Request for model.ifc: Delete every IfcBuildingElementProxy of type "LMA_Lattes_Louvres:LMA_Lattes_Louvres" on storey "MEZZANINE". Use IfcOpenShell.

First a look at what the model holds.

```python
import ifcopenshell
import ifcopenshell.util.element

model = ifcopenshell.open("model.ifc")
print(model.schema)
storey = next(s for s in model.by_type("IfcBuildingStorey") if s.Name == "MEZZANINE")
proxies = [e for e in ifcopenshell.util.element.get_decomposition(storey) if e.is_a("IfcBuildingElementProxy")]
seen = {}
for e in proxies:
    element_type = ifcopenshell.util.element.get_type(e)
    name = element_type.Name if element_type not in (None, e) else None
    seen[name] = seen.get(name, 0) + 1
for name, count in sorted(seen.items(), key=str):
    print(count, "x", name)
```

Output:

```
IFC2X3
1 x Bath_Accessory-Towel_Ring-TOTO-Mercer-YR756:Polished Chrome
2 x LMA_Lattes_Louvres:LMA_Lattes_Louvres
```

```python
import ifcopenshell
import ifcopenshell.api.root
import ifcopenshell.util.element

model = ifcopenshell.open("model.ifc")

storey = next(s for s in model.by_type("IfcBuildingStorey") if s.Name == "MEZZANINE")
proxies = [e for e in ifcopenshell.util.element.get_decomposition(storey) if e.is_a("IfcBuildingElementProxy")]
targets = [e for e in proxies if (t := ifcopenshell.util.element.get_type(e)) not in (None, e) and t.Name == "LMA_Lattes_Louvres:LMA_Lattes_Louvres"]

for e in targets:
    ifcopenshell.api.root.remove_product(model, product=e)
print(len(targets), "removed")

model.write("model_edited.ifc")
```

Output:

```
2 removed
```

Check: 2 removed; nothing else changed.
